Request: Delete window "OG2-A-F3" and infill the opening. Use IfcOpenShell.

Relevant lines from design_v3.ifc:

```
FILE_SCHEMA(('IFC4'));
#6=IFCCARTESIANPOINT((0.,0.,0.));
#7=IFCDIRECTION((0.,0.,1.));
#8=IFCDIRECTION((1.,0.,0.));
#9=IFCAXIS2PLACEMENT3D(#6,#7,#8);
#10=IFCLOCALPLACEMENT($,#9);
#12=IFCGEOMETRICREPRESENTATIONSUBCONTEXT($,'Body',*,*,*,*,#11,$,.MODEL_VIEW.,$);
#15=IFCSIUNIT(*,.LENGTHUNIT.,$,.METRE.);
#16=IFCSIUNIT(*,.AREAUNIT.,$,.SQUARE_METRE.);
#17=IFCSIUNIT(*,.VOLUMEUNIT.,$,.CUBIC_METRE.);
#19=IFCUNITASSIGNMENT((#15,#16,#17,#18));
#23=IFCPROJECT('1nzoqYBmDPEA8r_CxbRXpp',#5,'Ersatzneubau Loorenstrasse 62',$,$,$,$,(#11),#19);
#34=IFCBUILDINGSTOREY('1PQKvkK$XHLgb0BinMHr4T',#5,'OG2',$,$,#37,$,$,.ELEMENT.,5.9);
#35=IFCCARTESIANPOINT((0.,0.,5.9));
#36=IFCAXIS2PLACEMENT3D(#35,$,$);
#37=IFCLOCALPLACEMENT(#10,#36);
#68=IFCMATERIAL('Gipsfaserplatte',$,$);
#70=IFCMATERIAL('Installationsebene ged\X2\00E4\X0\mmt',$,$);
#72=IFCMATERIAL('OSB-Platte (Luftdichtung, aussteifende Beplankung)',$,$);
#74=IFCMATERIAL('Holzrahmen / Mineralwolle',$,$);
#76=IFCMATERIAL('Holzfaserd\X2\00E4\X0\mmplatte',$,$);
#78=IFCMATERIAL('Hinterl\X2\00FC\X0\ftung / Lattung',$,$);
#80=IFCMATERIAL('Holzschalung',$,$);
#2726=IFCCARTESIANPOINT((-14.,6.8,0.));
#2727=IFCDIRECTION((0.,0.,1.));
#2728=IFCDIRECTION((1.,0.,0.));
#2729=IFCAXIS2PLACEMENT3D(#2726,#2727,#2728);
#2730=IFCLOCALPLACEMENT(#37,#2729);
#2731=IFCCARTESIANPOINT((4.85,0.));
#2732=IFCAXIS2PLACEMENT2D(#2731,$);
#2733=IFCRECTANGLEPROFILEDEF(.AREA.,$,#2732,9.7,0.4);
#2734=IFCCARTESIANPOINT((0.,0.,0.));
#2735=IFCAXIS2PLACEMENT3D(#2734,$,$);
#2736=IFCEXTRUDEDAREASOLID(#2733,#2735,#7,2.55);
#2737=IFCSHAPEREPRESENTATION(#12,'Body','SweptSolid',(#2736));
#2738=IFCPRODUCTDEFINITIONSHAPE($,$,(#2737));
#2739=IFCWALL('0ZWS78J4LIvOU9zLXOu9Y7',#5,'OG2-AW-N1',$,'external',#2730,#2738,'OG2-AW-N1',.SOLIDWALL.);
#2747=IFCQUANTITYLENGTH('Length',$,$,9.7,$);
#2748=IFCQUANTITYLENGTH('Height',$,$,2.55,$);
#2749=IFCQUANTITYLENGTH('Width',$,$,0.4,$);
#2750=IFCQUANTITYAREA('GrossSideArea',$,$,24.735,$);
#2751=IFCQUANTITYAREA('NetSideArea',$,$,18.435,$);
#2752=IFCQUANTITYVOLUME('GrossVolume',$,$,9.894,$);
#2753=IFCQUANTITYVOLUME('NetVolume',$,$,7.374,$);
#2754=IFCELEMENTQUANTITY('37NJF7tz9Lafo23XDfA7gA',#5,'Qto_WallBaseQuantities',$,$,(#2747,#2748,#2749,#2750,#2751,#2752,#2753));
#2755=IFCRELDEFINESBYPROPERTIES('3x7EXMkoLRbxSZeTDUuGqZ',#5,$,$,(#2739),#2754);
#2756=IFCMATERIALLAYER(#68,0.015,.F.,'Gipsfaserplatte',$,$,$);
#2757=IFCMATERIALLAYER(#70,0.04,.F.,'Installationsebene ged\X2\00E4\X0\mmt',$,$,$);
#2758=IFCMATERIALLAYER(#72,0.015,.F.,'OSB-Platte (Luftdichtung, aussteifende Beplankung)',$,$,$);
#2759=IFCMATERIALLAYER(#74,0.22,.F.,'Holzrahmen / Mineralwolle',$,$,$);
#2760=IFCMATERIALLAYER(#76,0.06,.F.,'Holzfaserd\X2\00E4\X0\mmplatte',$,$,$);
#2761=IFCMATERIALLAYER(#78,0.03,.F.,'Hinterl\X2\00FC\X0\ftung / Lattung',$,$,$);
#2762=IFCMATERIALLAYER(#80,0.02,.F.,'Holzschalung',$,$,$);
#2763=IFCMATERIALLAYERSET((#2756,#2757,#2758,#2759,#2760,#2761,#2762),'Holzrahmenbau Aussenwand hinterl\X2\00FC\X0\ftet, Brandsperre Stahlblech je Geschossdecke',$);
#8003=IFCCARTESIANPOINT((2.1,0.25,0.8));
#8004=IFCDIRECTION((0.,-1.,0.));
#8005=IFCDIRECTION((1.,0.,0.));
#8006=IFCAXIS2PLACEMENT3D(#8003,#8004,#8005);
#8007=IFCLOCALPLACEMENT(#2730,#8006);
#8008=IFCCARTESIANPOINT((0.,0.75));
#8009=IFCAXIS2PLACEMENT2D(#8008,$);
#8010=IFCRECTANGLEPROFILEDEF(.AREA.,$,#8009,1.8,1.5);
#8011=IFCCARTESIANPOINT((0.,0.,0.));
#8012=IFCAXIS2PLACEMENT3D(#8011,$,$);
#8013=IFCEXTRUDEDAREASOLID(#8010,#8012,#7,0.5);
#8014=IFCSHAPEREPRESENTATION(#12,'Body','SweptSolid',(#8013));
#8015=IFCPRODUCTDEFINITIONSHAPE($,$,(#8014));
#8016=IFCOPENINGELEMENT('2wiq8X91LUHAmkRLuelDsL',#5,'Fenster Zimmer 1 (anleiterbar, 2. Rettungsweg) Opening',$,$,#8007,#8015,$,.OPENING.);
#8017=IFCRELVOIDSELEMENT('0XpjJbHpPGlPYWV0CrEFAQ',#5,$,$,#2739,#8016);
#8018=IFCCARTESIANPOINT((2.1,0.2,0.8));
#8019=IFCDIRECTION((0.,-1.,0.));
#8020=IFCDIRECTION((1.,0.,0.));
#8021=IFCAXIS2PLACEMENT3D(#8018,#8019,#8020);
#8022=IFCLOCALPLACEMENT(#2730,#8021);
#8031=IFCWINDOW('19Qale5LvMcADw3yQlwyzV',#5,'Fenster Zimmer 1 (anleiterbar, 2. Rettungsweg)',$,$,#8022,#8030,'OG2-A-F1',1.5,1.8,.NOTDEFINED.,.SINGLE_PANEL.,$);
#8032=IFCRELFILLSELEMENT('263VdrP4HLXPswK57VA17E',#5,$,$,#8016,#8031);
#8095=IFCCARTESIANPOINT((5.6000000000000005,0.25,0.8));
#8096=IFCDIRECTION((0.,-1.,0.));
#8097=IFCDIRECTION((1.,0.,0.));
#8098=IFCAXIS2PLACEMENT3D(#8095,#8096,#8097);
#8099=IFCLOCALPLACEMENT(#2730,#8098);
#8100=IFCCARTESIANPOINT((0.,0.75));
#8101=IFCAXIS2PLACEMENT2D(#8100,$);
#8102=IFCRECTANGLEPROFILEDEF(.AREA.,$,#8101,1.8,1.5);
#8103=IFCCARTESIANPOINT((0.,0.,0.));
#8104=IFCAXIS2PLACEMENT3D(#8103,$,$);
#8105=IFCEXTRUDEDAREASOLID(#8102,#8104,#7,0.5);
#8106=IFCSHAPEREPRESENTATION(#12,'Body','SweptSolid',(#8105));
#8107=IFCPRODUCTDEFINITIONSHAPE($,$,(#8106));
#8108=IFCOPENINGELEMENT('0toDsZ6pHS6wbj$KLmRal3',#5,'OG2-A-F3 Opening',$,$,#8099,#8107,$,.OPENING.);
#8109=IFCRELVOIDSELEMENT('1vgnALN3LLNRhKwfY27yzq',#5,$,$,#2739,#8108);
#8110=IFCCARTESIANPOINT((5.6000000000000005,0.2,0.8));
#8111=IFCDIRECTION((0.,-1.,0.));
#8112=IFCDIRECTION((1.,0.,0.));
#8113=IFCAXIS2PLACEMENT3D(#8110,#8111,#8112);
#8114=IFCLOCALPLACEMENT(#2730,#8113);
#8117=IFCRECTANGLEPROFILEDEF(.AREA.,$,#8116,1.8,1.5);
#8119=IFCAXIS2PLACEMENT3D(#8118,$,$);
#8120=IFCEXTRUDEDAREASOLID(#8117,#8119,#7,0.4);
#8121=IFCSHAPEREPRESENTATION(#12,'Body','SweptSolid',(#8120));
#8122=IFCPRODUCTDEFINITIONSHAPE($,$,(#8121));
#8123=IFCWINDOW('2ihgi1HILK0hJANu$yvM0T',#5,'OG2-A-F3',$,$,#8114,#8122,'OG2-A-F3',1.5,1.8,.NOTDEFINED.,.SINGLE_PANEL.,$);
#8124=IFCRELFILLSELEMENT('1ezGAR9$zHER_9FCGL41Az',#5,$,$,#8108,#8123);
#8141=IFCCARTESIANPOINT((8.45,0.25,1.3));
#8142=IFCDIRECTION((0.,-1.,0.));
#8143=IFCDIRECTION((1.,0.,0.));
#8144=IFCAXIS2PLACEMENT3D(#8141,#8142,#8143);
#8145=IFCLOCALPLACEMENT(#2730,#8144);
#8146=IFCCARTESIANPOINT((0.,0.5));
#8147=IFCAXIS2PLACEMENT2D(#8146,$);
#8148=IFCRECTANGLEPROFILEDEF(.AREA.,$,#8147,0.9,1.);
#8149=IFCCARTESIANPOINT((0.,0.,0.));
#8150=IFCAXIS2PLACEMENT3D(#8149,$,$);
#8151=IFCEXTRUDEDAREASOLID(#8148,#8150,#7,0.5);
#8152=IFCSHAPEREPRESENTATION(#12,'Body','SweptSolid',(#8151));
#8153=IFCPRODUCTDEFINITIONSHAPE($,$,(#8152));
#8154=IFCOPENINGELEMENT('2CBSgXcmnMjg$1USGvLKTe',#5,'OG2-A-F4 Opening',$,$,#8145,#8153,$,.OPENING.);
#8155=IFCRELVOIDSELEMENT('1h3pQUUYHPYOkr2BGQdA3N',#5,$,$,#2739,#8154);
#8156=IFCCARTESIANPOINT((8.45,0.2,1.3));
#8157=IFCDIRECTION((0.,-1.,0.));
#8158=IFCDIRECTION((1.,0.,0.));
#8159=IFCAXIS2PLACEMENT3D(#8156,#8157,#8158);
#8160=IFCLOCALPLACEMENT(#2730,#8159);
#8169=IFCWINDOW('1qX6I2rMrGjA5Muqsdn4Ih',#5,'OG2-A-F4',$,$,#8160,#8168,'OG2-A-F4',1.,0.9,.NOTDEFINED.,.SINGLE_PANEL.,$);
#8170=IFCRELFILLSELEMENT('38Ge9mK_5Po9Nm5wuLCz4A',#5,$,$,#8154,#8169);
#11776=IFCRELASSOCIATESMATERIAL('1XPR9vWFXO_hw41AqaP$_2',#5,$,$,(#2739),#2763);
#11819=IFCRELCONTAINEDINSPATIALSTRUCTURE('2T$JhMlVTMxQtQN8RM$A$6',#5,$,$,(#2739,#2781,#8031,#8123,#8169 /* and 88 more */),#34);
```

```python
import ifcopenshell
import ifcopenshell.api.feature
import ifcopenshell.api.pset
import ifcopenshell.api.root
import ifcopenshell.geom
import ifcopenshell.util.element
import ifcopenshell.util.shape
import ifcopenshell.util.unit

model = ifcopenshell.open("design_v3.ifc")
area_scale = ifcopenshell.util.unit.calculate_unit_scale(model, "AREAUNIT")
volume_scale = ifcopenshell.util.unit.calculate_unit_scale(model, "VOLUMEUNIT")
settings = ifcopenshell.geom.settings()


def volume(element):
    """Net volume in cubic metres, openings subtracted."""
    shape = ifcopenshell.geom.create_shape(settings, element)
    return ifcopenshell.util.shape.get_volume(shape.geometry)


window = model.by_guid("2ihgi1HILK0hJANu$yvM0T")
opening = window.FillsVoids[0].RelatingOpeningElement
wall = opening.VoidsElements[0].RelatingBuildingElement
before = volume(wall)

ifcopenshell.api.root.remove_product(model, product=window)
ifcopenshell.api.feature.remove_feature(model, feature=opening)

after = volume(wall)
thickness = 0.4  # wall thickness in metres

# Update the wall's stored quantities.
qto = model.by_id(ifcopenshell.util.element.get_pset(wall, "Qto_WallBaseQuantities", should_inherit=False)["id"])
ifcopenshell.api.pset.edit_qto(model, qto=qto, properties={
    "NetSideArea": after / thickness / area_scale,
    "NetVolume": after / volume_scale,
})

print(f"wall volume {before:.3f} -> {after:.3f} m3")

model.write("design_v3_edited.ifc")
```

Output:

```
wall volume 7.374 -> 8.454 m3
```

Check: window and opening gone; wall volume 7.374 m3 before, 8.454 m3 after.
